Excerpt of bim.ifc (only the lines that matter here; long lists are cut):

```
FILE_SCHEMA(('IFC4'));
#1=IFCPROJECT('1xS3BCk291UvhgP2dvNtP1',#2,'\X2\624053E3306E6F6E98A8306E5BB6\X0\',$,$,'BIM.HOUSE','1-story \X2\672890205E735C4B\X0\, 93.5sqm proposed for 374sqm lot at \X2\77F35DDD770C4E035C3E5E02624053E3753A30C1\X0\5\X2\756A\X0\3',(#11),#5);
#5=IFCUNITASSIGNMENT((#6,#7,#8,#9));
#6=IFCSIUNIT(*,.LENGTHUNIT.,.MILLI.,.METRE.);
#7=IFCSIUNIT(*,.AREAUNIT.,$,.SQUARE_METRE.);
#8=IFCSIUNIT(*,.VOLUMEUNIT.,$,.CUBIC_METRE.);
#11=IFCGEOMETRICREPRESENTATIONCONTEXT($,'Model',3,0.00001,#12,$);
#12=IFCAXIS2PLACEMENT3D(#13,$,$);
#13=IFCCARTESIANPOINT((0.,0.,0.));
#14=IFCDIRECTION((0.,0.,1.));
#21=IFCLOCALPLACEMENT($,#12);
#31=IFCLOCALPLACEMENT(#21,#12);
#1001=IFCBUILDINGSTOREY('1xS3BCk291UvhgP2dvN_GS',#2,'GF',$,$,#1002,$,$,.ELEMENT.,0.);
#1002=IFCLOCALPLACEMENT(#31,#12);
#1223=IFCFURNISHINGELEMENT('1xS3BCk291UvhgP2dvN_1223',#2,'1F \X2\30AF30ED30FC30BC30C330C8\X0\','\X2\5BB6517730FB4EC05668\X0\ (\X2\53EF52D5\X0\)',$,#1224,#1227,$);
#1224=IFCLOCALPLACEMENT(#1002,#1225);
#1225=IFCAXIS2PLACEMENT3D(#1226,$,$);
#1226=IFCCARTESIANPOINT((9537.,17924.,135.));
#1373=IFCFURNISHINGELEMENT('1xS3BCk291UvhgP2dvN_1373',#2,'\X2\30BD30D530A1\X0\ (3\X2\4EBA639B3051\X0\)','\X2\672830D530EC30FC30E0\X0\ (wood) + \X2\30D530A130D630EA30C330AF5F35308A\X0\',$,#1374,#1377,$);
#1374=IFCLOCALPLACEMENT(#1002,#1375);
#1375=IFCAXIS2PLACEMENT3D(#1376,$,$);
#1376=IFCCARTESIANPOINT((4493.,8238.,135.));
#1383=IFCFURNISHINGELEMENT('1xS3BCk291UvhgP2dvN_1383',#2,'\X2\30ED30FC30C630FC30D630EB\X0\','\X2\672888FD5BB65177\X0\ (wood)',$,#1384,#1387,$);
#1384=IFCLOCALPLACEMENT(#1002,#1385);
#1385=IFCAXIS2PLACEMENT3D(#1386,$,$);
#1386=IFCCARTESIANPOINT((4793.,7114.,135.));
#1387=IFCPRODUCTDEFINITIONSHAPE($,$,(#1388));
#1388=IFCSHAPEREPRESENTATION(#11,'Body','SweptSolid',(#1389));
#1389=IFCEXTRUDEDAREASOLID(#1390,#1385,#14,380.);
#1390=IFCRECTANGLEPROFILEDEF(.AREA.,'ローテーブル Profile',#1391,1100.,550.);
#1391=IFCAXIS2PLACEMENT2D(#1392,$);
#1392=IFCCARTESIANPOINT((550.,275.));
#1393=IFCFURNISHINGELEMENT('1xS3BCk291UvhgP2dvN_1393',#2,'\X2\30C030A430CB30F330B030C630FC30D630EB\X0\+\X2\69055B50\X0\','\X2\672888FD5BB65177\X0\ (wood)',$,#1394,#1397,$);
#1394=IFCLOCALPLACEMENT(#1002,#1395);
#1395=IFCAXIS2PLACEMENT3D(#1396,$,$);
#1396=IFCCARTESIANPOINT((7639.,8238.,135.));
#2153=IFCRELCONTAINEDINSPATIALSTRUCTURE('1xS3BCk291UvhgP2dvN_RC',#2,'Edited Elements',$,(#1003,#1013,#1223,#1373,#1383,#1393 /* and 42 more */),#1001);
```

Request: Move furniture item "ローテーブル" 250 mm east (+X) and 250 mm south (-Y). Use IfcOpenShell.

```python
import ifcopenshell
import ifcopenshell.api.geometry
import ifcopenshell.util.placement
import ifcopenshell.util.unit

model = ifcopenshell.open("bim.ifc")
unit_scale = ifcopenshell.util.unit.calculate_unit_scale(model)

item = model.by_guid("1xS3BCk291UvhgP2dvN_1383")
matrix = ifcopenshell.util.placement.get_local_placement(item.ObjectPlacement)
matrix[0, 3] += 0.25 / unit_scale
matrix[1, 3] -= 0.25 / unit_scale
ifcopenshell.api.geometry.edit_object_placement(model, product=item, matrix=matrix, is_si=False)

print(ifcopenshell.util.placement.get_local_placement(item.ObjectPlacement).round(3) + 0.0)

model.write("bim_edited.ifc")
```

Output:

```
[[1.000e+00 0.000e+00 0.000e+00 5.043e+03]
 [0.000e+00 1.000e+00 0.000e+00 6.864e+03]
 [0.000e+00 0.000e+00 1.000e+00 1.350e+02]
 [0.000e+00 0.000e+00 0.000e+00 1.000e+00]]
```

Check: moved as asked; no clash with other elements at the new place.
